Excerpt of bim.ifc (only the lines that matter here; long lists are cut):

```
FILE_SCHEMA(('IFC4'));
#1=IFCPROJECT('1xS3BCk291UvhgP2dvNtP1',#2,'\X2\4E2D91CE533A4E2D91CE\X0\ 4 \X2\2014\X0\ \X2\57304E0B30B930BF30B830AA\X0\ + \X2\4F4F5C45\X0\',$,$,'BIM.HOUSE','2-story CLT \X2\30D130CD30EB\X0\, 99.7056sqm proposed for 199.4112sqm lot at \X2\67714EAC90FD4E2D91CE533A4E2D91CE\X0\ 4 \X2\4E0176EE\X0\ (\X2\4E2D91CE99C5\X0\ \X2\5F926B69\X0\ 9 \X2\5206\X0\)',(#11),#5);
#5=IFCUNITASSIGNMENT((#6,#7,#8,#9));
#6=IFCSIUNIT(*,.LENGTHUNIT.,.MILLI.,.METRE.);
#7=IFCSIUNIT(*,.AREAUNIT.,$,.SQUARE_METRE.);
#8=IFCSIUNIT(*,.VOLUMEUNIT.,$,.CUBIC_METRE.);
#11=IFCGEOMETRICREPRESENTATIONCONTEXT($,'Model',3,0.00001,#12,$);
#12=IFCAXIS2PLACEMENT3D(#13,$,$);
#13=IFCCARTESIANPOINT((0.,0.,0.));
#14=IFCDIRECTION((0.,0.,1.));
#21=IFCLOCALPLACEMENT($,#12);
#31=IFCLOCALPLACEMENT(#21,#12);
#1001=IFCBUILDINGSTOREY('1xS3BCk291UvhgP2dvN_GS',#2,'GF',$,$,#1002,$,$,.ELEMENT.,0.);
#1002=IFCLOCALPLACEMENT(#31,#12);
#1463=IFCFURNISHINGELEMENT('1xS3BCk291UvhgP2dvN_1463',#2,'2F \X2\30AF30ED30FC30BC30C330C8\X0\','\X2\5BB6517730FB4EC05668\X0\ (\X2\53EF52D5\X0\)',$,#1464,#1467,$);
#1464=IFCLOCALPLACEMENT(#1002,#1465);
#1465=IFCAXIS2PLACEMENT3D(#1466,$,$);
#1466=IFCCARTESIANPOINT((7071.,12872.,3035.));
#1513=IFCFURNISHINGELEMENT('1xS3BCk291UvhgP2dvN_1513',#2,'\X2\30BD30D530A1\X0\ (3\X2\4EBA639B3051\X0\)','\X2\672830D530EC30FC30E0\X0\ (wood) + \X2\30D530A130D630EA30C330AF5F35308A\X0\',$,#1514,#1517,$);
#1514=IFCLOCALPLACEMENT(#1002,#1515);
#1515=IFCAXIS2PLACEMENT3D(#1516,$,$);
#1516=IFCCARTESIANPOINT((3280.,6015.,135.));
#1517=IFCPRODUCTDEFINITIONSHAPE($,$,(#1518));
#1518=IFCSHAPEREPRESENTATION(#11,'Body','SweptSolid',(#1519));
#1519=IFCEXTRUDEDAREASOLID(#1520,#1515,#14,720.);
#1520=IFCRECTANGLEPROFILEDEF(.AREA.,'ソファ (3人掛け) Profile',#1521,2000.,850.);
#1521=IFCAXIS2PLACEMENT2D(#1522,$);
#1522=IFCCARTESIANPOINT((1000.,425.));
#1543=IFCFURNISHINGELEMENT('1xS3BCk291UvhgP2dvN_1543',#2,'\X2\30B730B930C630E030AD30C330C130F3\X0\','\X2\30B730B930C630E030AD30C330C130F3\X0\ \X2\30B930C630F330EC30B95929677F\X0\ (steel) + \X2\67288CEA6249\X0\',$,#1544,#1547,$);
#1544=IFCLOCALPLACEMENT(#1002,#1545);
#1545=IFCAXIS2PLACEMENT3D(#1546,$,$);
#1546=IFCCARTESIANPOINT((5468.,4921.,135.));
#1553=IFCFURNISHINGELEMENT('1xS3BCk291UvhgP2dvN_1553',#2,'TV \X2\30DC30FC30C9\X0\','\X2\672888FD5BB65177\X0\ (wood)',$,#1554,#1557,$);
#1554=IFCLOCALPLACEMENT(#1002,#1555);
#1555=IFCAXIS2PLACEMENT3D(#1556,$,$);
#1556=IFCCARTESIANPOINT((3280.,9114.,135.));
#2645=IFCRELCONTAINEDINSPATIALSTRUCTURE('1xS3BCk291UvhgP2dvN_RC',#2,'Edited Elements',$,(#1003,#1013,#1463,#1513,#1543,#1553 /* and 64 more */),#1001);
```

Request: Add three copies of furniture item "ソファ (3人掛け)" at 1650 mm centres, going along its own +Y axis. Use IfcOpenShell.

```python
import ifcopenshell
import ifcopenshell.api.geometry
import ifcopenshell.api.root
import ifcopenshell.util.element
import ifcopenshell.util.placement
import ifcopenshell.util.unit

model = ifcopenshell.open("bim.ifc")
unit_scale = ifcopenshell.util.unit.calculate_unit_scale(model)


def reuse_history(source, copy):
    """copy_class also copies each property set's owner history, people and application; keep the originals."""
    for rel in copy.IsDefinedBy:
        if rel.is_a("IfcRelDefinesByProperties") and (history := rel.RelatingPropertyDefinition.OwnerHistory):
            rel.RelatingPropertyDefinition.OwnerHistory = source.OwnerHistory
            ifcopenshell.util.element.remove_deep2(model, history)


source = model.by_id(1513)
base = ifcopenshell.util.placement.get_local_placement(source.ObjectPlacement)
step = base[:3, 1] * 1.65 / unit_scale

for i in range(1, 4):
    copy = ifcopenshell.api.root.copy_class(model, product=source)
    copy.Representation = ifcopenshell.util.element.copy_deep(
        model, source.Representation, exclude=["IfcGeometricRepresentationContext", "IfcRepresentationMap"]
    )
    reuse_history(source, copy)
    matrix = base.copy()
    matrix[:3, 3] += i * step
    print("added at", matrix[:3, 3].round(3) + 0.0)
    ifcopenshell.api.geometry.edit_object_placement(model, product=copy, matrix=matrix, is_si=False)

model.write("bim_edited.ifc")
```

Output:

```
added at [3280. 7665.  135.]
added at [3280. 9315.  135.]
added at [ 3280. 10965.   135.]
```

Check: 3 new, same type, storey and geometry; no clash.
